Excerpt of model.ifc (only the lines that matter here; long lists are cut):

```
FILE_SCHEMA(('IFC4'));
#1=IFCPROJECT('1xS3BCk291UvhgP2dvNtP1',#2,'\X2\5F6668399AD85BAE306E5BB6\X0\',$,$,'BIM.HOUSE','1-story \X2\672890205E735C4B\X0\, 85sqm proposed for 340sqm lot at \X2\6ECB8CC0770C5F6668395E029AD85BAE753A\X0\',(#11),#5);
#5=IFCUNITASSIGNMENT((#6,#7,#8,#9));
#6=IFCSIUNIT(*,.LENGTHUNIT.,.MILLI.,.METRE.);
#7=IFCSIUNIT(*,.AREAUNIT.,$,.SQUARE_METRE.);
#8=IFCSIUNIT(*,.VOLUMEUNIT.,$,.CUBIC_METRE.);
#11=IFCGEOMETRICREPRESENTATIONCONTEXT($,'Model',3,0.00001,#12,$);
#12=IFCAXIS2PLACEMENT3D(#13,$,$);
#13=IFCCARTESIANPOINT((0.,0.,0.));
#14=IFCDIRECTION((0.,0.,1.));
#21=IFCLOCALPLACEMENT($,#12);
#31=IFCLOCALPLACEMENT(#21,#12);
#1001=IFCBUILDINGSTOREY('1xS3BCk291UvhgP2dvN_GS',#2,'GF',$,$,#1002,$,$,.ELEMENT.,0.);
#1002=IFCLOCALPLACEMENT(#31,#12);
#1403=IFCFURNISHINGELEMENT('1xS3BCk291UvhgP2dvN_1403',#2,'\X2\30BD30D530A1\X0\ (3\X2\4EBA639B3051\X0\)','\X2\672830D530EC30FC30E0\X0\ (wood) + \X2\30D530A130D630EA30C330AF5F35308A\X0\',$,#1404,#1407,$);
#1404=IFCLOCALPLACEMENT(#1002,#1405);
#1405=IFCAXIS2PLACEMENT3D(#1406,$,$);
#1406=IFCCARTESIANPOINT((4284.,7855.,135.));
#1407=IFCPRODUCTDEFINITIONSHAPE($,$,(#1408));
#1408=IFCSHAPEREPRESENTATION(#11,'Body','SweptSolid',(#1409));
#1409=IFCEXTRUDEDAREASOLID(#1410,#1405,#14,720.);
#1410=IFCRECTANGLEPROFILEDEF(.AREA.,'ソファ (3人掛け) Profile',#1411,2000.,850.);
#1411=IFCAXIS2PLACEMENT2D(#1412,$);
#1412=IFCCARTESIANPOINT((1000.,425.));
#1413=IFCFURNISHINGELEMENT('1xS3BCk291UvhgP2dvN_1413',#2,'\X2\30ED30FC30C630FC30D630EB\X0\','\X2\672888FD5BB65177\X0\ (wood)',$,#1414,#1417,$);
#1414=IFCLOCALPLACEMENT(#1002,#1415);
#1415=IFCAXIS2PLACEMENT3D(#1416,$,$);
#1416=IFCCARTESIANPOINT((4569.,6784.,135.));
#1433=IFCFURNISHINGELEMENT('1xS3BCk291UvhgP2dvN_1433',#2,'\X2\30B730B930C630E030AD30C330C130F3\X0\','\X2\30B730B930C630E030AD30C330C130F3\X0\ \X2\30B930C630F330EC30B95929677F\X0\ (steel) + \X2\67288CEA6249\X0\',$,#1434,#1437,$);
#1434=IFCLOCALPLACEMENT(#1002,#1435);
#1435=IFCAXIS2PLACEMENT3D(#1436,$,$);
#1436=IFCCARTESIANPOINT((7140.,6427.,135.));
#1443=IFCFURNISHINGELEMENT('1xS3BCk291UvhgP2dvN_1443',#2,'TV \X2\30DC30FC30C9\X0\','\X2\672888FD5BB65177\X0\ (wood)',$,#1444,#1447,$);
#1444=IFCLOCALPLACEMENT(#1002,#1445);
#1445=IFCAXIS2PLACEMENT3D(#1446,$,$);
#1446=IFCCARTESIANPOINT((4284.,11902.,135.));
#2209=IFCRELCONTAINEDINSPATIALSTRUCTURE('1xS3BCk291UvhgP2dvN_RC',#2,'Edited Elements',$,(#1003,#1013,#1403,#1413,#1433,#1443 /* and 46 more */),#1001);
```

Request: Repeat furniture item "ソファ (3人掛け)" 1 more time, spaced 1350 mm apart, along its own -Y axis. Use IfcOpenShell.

```python
import ifcopenshell
import ifcopenshell.api.geometry
import ifcopenshell.api.root
import ifcopenshell.util.element
import ifcopenshell.util.placement
import ifcopenshell.util.unit

model = ifcopenshell.open("model.ifc")
unit_scale = ifcopenshell.util.unit.calculate_unit_scale(model)


def reuse_history(source, copy):
    """copy_class also copies each property set's owner history, people and application; keep the originals."""
    for rel in copy.IsDefinedBy:
        if rel.is_a("IfcRelDefinesByProperties") and (history := rel.RelatingPropertyDefinition.OwnerHistory):
            rel.RelatingPropertyDefinition.OwnerHistory = source.OwnerHistory
            ifcopenshell.util.element.remove_deep2(model, history)


source = model.by_id(1403)
base = ifcopenshell.util.placement.get_local_placement(source.ObjectPlacement)
step = -base[:3, 1] * 1.35 / unit_scale

for i in range(1, 2):
    copy = ifcopenshell.api.root.copy_class(model, product=source)
    copy.Representation = ifcopenshell.util.element.copy_deep(
        model, source.Representation, exclude=["IfcGeometricRepresentationContext", "IfcRepresentationMap"]
    )
    reuse_history(source, copy)
    matrix = base.copy()
    matrix[:3, 3] += i * step
    print("added at", matrix[:3, 3].round(3) + 0.0)
    ifcopenshell.api.geometry.edit_object_placement(model, product=copy, matrix=matrix, is_si=False)

model.write("model-out.ifc")
```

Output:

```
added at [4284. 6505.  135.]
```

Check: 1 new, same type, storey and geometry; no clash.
